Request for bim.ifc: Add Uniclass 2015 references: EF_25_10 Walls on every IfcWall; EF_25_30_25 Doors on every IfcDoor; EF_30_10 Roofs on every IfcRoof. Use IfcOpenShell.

First a look at what the model holds.

```python
import ifcopenshell

model = ifcopenshell.open("bim.ifc")
print(model.schema)
print("classifications:", [c.Name for c in model.by_type("IfcClassification")])
for ifc_class in ("IfcDoor", "IfcRoof", "IfcStair", "IfcWall", "IfcWindow"):
    print(ifc_class, len(model.by_type(ifc_class)))
```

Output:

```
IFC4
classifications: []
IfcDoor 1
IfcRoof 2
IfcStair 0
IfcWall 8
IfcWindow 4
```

```python
import ifcopenshell
import ifcopenshell.api.classification

model = ifcopenshell.open("bim.ifc")

system = ifcopenshell.api.classification.add_classification(model, classification="Uniclass 2015")

codes = {
    "IfcWall": ("EF_25_10", "Walls"),
    "IfcDoor": ("EF_25_30_25", "Doors"),
    "IfcRoof": ("EF_30_10", "Roofs"),
}
for ifc_class, (code, name) in codes.items():
    products = model.by_type(ifc_class)
    ifcopenshell.api.classification.add_reference(
        model, products=products, classification=system, identification=code, name=name
    )
    print(code, len(products))

model.write("bim_v2.ifc")
```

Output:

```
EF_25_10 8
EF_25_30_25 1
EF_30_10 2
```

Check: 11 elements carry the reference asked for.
